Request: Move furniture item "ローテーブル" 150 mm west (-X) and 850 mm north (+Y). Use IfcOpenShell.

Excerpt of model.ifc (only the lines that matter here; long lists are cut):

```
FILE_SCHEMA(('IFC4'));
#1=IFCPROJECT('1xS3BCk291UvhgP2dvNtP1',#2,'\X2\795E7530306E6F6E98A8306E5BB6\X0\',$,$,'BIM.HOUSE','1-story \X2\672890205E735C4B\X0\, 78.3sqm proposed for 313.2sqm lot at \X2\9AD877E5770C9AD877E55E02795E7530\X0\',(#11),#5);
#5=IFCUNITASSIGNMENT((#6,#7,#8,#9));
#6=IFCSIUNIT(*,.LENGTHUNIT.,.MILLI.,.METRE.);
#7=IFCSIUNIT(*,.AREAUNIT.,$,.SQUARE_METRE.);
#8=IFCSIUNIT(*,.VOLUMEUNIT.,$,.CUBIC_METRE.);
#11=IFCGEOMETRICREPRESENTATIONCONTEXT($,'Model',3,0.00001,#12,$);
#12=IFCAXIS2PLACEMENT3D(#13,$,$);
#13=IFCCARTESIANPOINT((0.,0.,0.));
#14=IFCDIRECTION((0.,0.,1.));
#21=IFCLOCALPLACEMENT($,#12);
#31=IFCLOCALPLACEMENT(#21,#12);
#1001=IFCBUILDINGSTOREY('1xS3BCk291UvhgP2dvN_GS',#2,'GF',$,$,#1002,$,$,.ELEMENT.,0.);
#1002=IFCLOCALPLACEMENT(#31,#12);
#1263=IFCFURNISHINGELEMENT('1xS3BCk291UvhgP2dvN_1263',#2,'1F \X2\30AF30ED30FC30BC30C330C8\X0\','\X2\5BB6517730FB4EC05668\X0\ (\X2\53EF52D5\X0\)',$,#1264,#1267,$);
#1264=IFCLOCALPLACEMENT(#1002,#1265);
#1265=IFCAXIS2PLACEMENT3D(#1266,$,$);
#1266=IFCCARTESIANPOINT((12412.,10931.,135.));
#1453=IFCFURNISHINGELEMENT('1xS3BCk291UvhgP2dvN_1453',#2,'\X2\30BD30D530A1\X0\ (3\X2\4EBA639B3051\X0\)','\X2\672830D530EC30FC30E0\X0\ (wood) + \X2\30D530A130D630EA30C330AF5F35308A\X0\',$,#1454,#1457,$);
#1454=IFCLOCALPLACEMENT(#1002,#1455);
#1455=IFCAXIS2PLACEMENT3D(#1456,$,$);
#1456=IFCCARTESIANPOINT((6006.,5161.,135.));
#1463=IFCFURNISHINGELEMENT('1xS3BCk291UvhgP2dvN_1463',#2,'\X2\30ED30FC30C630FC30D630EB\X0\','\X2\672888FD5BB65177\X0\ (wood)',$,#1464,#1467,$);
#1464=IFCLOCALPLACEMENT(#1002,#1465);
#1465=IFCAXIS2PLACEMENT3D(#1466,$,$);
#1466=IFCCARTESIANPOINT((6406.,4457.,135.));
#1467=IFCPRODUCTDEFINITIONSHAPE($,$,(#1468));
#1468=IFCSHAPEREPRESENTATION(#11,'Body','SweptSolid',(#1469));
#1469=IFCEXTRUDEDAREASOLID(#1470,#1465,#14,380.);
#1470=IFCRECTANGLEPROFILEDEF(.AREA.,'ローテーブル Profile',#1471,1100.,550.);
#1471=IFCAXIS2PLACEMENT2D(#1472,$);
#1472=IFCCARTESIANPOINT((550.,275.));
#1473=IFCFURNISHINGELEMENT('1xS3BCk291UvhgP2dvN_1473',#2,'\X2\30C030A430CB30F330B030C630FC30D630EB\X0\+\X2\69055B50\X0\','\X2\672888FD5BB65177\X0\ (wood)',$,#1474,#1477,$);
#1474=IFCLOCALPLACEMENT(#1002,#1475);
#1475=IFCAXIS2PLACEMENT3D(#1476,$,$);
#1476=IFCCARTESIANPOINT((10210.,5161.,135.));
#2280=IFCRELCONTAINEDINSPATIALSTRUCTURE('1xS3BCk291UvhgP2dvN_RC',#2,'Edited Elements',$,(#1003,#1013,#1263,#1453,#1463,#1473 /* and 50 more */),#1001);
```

```python
import ifcopenshell
import ifcopenshell.api.geometry
import ifcopenshell.util.placement
import ifcopenshell.util.unit

model = ifcopenshell.open("model.ifc")
unit_scale = ifcopenshell.util.unit.calculate_unit_scale(model)

item = model.by_id(1463)
matrix = ifcopenshell.util.placement.get_local_placement(item.ObjectPlacement)
matrix[0, 3] -= 0.15 / unit_scale
matrix[1, 3] += 0.85 / unit_scale
ifcopenshell.api.geometry.edit_object_placement(model, product=item, matrix=matrix, is_si=False)

print(ifcopenshell.util.placement.get_local_placement(item.ObjectPlacement).round(3) + 0.0)

model.write("model_v2.ifc")
```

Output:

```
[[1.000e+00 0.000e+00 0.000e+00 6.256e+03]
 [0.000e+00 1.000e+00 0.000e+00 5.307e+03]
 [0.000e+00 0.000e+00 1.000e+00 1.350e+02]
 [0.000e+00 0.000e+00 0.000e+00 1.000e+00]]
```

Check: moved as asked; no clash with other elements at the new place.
